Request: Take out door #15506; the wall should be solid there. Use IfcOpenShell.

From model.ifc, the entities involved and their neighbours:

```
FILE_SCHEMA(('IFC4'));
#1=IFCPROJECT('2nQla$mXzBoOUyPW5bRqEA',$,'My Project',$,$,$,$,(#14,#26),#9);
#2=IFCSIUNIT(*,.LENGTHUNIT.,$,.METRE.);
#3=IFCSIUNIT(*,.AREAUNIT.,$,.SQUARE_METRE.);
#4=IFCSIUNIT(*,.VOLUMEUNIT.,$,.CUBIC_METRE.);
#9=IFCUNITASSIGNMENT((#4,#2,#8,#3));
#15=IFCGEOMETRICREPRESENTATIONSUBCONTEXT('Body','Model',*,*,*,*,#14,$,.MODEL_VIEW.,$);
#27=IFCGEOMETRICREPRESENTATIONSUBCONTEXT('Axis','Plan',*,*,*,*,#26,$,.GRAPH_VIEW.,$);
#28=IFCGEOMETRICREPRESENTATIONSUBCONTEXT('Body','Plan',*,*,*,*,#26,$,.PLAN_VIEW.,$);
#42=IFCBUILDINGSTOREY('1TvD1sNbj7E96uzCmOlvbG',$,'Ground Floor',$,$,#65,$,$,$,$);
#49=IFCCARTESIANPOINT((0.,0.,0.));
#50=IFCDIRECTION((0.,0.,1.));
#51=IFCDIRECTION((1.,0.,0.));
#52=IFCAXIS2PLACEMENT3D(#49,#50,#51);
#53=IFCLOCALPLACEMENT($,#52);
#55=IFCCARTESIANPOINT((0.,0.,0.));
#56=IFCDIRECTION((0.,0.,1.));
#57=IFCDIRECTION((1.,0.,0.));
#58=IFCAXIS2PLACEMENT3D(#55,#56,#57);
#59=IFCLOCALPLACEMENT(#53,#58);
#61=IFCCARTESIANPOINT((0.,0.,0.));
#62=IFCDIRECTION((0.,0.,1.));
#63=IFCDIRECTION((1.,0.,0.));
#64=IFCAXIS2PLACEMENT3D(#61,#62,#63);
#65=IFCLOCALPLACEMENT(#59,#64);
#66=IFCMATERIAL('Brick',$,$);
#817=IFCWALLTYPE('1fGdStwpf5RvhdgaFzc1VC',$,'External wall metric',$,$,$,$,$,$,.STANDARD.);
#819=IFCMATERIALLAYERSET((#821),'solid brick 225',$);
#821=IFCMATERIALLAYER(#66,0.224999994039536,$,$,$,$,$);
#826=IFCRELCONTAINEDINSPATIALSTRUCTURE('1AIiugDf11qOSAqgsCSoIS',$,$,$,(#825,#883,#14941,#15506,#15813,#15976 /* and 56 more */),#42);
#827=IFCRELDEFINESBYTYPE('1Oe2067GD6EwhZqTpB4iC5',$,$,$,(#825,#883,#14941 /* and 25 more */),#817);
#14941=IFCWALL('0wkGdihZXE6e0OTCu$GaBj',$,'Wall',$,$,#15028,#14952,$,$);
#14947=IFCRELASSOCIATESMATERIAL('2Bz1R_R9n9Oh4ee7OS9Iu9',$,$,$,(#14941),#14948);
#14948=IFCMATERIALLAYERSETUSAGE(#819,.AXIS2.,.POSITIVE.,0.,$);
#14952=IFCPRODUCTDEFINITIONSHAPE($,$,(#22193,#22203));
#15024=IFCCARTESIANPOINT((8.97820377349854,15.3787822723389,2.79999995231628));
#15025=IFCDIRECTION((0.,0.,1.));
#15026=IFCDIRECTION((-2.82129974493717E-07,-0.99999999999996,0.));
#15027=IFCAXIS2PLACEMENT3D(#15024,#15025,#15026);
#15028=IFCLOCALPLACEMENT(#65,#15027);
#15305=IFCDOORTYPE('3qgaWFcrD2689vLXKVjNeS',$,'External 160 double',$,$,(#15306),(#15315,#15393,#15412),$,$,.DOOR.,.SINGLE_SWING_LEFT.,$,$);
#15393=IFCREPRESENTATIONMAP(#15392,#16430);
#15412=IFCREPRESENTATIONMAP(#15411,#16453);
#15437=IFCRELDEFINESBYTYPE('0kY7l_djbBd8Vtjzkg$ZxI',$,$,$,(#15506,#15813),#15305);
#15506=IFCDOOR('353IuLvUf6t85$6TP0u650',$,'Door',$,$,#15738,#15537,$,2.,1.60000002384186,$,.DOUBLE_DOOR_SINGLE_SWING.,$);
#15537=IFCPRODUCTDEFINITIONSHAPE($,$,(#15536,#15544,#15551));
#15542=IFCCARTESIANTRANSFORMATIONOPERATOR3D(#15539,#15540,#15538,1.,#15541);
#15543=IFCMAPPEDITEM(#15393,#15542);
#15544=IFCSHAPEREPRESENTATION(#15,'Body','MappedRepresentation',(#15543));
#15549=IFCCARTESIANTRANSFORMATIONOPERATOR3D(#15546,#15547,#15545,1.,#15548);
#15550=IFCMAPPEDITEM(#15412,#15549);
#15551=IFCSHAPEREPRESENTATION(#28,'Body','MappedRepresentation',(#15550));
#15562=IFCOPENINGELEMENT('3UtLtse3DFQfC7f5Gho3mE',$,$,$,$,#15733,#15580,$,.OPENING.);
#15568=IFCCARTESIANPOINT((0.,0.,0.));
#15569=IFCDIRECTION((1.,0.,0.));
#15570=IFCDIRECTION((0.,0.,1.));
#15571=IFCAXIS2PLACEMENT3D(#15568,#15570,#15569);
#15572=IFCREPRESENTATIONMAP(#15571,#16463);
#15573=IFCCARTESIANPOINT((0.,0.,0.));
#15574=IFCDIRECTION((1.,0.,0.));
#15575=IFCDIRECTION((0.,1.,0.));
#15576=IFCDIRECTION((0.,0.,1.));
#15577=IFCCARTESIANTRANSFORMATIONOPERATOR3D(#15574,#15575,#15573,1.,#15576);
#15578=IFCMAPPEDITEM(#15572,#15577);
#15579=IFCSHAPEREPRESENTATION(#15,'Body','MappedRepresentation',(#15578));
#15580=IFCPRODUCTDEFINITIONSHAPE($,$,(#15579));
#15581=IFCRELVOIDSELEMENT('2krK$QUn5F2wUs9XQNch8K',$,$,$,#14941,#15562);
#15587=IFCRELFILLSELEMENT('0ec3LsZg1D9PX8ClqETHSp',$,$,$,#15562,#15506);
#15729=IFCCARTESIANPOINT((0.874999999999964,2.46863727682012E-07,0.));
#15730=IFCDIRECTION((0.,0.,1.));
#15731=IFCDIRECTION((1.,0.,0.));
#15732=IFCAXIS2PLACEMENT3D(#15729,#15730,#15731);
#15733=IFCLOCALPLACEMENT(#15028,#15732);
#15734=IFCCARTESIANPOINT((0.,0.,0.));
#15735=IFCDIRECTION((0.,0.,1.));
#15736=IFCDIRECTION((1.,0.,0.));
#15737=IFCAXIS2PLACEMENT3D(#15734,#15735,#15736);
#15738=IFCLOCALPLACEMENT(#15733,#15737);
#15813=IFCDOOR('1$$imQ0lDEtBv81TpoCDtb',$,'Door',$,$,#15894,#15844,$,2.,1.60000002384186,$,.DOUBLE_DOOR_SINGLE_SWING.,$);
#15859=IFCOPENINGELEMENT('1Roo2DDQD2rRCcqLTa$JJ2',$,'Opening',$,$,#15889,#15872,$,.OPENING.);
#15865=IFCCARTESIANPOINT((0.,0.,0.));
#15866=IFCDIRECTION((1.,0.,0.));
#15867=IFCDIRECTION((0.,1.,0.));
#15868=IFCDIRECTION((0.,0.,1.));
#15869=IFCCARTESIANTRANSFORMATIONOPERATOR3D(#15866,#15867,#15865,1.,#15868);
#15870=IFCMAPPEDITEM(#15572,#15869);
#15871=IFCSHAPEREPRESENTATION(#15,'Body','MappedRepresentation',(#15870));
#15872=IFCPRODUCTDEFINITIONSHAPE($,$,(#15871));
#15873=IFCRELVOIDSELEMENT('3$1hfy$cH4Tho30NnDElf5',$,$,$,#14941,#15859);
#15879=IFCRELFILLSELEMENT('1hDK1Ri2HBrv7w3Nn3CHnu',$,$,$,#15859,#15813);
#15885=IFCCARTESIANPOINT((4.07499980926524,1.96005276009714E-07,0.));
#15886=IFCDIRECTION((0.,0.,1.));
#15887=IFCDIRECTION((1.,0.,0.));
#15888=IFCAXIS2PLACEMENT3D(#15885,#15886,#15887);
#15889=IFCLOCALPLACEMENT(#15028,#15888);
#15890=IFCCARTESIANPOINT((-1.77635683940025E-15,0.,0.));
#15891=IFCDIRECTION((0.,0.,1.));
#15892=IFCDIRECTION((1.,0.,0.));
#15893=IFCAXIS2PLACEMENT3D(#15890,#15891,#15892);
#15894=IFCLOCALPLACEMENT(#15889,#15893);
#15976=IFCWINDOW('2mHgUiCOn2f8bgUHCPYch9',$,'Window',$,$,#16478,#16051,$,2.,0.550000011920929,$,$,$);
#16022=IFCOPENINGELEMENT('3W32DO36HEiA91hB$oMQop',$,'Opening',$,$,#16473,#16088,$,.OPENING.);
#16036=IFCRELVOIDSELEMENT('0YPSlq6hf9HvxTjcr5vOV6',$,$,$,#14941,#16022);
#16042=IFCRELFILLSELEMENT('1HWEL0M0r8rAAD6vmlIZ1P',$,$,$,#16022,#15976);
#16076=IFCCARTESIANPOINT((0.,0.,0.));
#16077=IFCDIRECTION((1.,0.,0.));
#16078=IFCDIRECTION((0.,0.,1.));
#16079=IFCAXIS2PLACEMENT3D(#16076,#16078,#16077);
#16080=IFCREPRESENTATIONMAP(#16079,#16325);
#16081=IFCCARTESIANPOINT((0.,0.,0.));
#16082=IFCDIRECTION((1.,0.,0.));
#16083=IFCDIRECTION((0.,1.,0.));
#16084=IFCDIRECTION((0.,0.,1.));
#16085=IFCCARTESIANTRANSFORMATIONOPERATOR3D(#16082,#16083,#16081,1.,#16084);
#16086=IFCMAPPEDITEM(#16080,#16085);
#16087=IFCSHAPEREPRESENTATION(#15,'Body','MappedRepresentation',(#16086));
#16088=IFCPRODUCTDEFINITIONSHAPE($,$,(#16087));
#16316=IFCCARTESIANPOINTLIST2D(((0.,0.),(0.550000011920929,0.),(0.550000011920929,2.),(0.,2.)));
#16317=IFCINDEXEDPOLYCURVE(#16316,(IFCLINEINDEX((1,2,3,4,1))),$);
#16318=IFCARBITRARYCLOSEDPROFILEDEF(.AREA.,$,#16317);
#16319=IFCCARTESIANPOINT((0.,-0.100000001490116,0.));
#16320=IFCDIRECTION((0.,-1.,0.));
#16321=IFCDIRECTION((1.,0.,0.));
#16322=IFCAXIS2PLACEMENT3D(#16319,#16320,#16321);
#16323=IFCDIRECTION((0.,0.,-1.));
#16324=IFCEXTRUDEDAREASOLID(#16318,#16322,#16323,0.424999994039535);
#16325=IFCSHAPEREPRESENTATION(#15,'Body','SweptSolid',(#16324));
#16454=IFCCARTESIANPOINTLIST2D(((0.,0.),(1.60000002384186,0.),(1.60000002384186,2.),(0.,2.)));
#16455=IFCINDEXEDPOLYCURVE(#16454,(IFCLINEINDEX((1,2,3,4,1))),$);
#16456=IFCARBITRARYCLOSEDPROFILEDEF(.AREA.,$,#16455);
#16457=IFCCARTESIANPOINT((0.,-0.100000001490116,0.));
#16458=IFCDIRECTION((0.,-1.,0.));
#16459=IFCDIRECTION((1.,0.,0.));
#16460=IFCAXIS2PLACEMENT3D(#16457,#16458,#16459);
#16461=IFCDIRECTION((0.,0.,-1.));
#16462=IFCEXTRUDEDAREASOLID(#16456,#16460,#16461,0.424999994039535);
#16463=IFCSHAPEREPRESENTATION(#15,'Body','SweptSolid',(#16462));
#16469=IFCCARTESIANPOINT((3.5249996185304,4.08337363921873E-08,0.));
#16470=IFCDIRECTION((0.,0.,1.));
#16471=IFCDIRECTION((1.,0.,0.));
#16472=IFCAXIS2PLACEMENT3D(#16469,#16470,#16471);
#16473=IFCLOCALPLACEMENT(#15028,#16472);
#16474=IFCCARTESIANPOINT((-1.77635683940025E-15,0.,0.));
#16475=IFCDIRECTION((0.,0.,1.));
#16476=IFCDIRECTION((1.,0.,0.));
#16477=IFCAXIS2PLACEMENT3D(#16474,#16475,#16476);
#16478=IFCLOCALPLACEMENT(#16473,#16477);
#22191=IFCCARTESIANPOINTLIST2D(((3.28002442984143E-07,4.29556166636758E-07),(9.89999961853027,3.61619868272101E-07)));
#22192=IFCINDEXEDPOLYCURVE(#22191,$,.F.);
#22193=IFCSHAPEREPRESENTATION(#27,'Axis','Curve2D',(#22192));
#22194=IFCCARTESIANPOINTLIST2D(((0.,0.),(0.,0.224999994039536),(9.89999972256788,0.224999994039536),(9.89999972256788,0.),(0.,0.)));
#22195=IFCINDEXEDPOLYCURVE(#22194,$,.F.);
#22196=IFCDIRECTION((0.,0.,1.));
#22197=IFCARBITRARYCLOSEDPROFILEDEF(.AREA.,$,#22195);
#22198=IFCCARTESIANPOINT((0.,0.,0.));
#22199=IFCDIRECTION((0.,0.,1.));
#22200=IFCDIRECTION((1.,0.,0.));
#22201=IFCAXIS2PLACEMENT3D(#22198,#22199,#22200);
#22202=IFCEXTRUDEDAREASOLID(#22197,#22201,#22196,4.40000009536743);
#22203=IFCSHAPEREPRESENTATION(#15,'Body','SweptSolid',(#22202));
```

```python
import ifcopenshell
import ifcopenshell.api.feature
import ifcopenshell.api.root
import ifcopenshell.geom
import ifcopenshell.util.shape

model = ifcopenshell.open("model.ifc")
settings = ifcopenshell.geom.settings()


def volume(element):
    """Net volume in cubic metres, openings subtracted."""
    shape = ifcopenshell.geom.create_shape(settings, element)
    return ifcopenshell.util.shape.get_volume(shape.geometry)


door = model.by_id(15506)
opening = door.FillsVoids[0].RelatingOpeningElement
wall = opening.VoidsElements[0].RelatingBuildingElement
before = volume(wall)

ifcopenshell.api.root.remove_product(model, product=door)
ifcopenshell.api.feature.remove_feature(model, feature=opening)

after = volume(wall)

print(f"wall volume {before:.3f} -> {after:.3f} m3")

model.write("model_rev.ifc")
```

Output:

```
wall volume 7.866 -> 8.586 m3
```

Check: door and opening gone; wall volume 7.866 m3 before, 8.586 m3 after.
